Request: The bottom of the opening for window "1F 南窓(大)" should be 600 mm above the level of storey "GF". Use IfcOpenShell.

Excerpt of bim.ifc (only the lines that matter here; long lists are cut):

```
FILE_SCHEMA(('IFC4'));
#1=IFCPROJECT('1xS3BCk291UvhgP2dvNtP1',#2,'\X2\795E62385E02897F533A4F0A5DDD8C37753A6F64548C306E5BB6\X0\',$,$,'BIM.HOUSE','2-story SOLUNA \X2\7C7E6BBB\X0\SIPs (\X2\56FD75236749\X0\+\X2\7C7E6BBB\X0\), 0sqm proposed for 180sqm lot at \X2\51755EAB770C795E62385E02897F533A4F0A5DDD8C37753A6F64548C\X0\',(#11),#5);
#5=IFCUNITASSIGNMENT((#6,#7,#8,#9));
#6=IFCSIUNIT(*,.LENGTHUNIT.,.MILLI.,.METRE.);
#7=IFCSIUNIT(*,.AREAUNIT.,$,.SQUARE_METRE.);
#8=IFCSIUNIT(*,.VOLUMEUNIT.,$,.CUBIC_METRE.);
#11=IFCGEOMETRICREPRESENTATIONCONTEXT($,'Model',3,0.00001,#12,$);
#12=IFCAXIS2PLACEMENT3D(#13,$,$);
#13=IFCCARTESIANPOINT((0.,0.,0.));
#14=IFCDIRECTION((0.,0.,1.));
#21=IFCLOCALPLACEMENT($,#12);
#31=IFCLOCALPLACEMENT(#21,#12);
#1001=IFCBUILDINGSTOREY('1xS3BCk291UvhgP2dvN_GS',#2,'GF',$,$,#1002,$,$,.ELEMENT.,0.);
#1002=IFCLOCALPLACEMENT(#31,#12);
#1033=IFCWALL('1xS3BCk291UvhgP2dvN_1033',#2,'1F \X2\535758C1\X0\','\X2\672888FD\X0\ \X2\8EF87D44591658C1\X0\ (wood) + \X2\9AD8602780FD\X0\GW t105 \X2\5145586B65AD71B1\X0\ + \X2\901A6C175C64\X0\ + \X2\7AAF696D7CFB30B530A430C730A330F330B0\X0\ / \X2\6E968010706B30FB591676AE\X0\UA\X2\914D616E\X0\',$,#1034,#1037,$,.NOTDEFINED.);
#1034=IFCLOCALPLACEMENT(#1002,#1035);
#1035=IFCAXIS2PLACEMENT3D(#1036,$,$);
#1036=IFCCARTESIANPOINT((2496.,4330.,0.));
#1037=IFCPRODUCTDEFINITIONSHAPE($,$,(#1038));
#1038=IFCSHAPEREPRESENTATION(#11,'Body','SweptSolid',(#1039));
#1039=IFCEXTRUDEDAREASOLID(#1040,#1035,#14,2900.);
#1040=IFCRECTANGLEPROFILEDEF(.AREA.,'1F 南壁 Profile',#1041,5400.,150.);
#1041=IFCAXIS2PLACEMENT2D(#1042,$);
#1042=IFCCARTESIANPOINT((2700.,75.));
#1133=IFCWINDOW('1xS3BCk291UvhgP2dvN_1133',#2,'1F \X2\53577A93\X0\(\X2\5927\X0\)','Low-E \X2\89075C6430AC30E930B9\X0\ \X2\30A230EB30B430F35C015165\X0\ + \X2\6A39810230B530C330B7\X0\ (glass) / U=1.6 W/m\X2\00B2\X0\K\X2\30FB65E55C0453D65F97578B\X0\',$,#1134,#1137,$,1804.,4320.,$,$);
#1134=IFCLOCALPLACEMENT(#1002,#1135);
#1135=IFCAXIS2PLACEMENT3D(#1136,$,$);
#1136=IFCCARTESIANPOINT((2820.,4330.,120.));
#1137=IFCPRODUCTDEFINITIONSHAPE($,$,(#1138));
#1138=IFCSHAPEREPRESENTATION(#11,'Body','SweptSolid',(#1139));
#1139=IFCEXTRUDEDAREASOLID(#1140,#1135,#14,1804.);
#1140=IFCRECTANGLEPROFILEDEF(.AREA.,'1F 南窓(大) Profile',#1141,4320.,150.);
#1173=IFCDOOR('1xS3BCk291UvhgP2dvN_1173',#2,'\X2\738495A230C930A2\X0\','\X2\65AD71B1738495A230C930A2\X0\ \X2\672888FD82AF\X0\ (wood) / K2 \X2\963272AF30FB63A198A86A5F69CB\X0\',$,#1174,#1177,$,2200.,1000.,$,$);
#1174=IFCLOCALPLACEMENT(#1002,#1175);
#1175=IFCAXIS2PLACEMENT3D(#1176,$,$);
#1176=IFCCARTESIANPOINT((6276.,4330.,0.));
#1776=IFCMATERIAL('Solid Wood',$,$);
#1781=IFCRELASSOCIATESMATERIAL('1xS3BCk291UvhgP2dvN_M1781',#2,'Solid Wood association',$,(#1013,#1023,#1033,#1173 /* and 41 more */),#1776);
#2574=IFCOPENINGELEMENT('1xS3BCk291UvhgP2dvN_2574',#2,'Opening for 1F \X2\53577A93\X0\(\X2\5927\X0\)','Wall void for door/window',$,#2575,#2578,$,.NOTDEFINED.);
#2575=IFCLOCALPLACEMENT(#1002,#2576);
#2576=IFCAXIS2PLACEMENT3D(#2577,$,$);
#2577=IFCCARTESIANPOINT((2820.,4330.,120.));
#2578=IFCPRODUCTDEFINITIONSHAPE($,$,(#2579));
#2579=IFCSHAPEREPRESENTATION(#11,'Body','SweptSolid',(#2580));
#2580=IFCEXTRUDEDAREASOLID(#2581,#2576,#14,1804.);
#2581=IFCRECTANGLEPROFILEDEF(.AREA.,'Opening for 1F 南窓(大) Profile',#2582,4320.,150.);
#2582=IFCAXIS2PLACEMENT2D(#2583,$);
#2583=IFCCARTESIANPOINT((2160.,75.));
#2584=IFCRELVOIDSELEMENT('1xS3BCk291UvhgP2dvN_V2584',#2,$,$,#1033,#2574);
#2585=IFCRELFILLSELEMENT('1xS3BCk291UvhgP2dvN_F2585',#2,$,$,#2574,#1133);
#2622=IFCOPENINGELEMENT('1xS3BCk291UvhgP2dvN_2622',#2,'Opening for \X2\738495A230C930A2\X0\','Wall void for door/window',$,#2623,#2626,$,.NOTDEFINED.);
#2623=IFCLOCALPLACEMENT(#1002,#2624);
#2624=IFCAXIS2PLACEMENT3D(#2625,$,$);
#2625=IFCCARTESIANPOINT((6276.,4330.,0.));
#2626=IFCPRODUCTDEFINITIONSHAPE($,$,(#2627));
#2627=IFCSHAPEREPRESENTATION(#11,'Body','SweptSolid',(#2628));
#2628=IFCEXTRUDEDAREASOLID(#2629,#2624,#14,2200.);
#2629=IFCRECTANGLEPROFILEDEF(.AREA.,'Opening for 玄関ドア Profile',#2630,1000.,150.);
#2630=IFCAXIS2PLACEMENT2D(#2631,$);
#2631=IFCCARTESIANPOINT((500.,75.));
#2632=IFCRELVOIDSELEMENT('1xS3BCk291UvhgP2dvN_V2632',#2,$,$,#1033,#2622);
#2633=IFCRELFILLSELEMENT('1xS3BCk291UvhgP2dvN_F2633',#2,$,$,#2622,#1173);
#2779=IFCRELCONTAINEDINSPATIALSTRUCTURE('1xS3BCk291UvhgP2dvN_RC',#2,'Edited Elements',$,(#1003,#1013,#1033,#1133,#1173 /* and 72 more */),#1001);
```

```python
import numpy as np
import ifcopenshell
import ifcopenshell.api.geometry
import ifcopenshell.geom
import ifcopenshell.util.element
import ifcopenshell.util.placement
import ifcopenshell.util.shape
import ifcopenshell.util.unit

model = ifcopenshell.open("bim.ifc")
unit_scale = ifcopenshell.util.unit.calculate_unit_scale(model)

window = model.by_guid("1xS3BCk291UvhgP2dvN_1133")
opening = window.FillsVoids[0].RelatingOpeningElement
storey = ifcopenshell.util.element.get_container(window, ifc_class="IfcBuildingStorey")
level = ifcopenshell.util.placement.get_local_placement(storey.ObjectPlacement)[2, 3]

# The opening's origin need not be at the sill, so measure its lowest point.
shape = ifcopenshell.geom.create_shape(ifcopenshell.geom.settings(), opening)
bottom = ifcopenshell.util.shape.get_shape_bottom_elevation(shape, shape.geometry) / unit_scale
dz = level + 0.6 / unit_scale - bottom

shift = np.array([0.0, 0.0, dz])
# The window is not placed relative to its opening, so move both.
for product in (opening, window):
    matrix = ifcopenshell.util.placement.get_local_placement(product.ObjectPlacement)
    matrix[:3, 3] += shift
    ifcopenshell.api.geometry.edit_object_placement(model, product=product, matrix=matrix, is_si=False)

print(f"moved by {dz * unit_scale:+.3f} m")

model.write("bim-out.ifc")
```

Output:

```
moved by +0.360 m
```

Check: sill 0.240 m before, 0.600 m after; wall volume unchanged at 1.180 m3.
